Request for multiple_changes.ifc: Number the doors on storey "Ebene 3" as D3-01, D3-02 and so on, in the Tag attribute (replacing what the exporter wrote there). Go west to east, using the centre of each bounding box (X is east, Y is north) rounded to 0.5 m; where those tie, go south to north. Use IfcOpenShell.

First a look at what the model holds.

```python
import ifcopenshell
import ifcopenshell.util.element
import ifcopenshell.util.placement

model = ifcopenshell.open("multiple_changes.ifc")
print(model.schema)
storey = next(s for s in model.by_type("IfcBuildingStorey") if s.Name == "Ebene 3")
doors = [e for e in ifcopenshell.util.element.get_decomposition(storey) if e.is_a("IfcDoor")]
for e in sorted(doors, key=lambda e: e.id()):
    origin = ifcopenshell.util.placement.get_local_placement(e.ObjectPlacement)[:3, 3]
    print(e.id(), e.Tag, e.Name, origin.round(2) + 0.0, sep=" | ")
```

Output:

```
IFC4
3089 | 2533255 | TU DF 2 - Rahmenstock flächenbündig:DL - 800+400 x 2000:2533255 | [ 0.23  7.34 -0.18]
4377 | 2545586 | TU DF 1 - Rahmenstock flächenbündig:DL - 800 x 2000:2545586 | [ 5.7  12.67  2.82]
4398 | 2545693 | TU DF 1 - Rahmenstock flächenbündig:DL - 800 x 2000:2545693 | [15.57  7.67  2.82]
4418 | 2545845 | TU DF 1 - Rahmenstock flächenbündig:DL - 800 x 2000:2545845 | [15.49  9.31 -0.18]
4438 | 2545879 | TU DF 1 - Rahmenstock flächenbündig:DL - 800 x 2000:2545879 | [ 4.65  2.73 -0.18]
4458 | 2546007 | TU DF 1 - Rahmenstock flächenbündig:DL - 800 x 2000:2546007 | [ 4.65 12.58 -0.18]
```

```python
import ifcopenshell
import ifcopenshell.geom
import ifcopenshell.util.element
import ifcopenshell.util.shape

model = ifcopenshell.open("multiple_changes.ifc")
settings = ifcopenshell.geom.settings()
settings.set("use-world-coords", True)


def centre(element):
    shape = ifcopenshell.geom.create_shape(settings, element)
    return ifcopenshell.util.shape.get_bbox_centroid(shape.geometry)


storey = next(s for s in model.by_type("IfcBuildingStorey") if s.Name == "Ebene 3")
doors = [e for e in ifcopenshell.util.element.get_decomposition(storey) if e.is_a("IfcDoor")]

# Insertion points can sit at a corner or the storey origin, so sort by the geometry (in metres).
centres = {e: centre(e) for e in doors}
doors.sort(key=lambda e: (round(centres[e][0] / 0.5), centres[e][1]))

for i, e in enumerate(doors, start=1):
    number = f"D3-{i:02d}"
    e.Tag = number
    print(e.id(), number)

model.write("multiple_changes_rev.ifc")
```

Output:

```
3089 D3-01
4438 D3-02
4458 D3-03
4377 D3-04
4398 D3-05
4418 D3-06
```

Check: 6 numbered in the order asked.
